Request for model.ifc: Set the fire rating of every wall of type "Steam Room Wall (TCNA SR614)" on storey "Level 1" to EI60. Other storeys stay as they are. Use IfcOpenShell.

First a look at what the model holds.

```python
import ifcopenshell
import ifcopenshell.util.element

model = ifcopenshell.open("model.ifc")
print(model.schema)
storey = next(s for s in model.by_type("IfcBuildingStorey") if s.Name == "Level 1")
walls = [e for e in ifcopenshell.util.element.get_decomposition(storey) if e.is_a("IfcWall")]
seen = {}
for e in walls:
    element_type = ifcopenshell.util.element.get_type(e)
    key = (element_type.Name if element_type != e and element_type else None, ifcopenshell.util.element.get_pset(e, "Pset_WallCommon", "FireRating"))
    seen[key] = seen.get(key, 0) + 1
for (name, value), count in sorted(seen.items(), key=str):
    print(count, "x", name, "|", value)
```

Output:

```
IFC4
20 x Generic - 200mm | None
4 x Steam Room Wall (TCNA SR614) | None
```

```python
import ifcopenshell
import ifcopenshell.api.pset
import ifcopenshell.util.element

model = ifcopenshell.open("model.ifc")

storey = next(s for s in model.by_type("IfcBuildingStorey") if s.Name == "Level 1")
walls = [e for e in ifcopenshell.util.element.get_decomposition(storey) if e.is_a("IfcWall")]

count = 0
for e in walls:
    element_type = ifcopenshell.util.element.get_type(e)
    if element_type in (None, e) or element_type.Name != "Steam Room Wall (TCNA SR614)":
        continue
    # add_pset returns the element's existing set when there is one.
    pset = ifcopenshell.api.pset.add_pset(model, product=e, name="Pset_WallCommon")
    ifcopenshell.api.pset.edit_pset(model, pset=pset, properties={"FireRating": "EI60"})
    count += 1

print(count, "walls updated")

model.write("model_v2.ifc")
```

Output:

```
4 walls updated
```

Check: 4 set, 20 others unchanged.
